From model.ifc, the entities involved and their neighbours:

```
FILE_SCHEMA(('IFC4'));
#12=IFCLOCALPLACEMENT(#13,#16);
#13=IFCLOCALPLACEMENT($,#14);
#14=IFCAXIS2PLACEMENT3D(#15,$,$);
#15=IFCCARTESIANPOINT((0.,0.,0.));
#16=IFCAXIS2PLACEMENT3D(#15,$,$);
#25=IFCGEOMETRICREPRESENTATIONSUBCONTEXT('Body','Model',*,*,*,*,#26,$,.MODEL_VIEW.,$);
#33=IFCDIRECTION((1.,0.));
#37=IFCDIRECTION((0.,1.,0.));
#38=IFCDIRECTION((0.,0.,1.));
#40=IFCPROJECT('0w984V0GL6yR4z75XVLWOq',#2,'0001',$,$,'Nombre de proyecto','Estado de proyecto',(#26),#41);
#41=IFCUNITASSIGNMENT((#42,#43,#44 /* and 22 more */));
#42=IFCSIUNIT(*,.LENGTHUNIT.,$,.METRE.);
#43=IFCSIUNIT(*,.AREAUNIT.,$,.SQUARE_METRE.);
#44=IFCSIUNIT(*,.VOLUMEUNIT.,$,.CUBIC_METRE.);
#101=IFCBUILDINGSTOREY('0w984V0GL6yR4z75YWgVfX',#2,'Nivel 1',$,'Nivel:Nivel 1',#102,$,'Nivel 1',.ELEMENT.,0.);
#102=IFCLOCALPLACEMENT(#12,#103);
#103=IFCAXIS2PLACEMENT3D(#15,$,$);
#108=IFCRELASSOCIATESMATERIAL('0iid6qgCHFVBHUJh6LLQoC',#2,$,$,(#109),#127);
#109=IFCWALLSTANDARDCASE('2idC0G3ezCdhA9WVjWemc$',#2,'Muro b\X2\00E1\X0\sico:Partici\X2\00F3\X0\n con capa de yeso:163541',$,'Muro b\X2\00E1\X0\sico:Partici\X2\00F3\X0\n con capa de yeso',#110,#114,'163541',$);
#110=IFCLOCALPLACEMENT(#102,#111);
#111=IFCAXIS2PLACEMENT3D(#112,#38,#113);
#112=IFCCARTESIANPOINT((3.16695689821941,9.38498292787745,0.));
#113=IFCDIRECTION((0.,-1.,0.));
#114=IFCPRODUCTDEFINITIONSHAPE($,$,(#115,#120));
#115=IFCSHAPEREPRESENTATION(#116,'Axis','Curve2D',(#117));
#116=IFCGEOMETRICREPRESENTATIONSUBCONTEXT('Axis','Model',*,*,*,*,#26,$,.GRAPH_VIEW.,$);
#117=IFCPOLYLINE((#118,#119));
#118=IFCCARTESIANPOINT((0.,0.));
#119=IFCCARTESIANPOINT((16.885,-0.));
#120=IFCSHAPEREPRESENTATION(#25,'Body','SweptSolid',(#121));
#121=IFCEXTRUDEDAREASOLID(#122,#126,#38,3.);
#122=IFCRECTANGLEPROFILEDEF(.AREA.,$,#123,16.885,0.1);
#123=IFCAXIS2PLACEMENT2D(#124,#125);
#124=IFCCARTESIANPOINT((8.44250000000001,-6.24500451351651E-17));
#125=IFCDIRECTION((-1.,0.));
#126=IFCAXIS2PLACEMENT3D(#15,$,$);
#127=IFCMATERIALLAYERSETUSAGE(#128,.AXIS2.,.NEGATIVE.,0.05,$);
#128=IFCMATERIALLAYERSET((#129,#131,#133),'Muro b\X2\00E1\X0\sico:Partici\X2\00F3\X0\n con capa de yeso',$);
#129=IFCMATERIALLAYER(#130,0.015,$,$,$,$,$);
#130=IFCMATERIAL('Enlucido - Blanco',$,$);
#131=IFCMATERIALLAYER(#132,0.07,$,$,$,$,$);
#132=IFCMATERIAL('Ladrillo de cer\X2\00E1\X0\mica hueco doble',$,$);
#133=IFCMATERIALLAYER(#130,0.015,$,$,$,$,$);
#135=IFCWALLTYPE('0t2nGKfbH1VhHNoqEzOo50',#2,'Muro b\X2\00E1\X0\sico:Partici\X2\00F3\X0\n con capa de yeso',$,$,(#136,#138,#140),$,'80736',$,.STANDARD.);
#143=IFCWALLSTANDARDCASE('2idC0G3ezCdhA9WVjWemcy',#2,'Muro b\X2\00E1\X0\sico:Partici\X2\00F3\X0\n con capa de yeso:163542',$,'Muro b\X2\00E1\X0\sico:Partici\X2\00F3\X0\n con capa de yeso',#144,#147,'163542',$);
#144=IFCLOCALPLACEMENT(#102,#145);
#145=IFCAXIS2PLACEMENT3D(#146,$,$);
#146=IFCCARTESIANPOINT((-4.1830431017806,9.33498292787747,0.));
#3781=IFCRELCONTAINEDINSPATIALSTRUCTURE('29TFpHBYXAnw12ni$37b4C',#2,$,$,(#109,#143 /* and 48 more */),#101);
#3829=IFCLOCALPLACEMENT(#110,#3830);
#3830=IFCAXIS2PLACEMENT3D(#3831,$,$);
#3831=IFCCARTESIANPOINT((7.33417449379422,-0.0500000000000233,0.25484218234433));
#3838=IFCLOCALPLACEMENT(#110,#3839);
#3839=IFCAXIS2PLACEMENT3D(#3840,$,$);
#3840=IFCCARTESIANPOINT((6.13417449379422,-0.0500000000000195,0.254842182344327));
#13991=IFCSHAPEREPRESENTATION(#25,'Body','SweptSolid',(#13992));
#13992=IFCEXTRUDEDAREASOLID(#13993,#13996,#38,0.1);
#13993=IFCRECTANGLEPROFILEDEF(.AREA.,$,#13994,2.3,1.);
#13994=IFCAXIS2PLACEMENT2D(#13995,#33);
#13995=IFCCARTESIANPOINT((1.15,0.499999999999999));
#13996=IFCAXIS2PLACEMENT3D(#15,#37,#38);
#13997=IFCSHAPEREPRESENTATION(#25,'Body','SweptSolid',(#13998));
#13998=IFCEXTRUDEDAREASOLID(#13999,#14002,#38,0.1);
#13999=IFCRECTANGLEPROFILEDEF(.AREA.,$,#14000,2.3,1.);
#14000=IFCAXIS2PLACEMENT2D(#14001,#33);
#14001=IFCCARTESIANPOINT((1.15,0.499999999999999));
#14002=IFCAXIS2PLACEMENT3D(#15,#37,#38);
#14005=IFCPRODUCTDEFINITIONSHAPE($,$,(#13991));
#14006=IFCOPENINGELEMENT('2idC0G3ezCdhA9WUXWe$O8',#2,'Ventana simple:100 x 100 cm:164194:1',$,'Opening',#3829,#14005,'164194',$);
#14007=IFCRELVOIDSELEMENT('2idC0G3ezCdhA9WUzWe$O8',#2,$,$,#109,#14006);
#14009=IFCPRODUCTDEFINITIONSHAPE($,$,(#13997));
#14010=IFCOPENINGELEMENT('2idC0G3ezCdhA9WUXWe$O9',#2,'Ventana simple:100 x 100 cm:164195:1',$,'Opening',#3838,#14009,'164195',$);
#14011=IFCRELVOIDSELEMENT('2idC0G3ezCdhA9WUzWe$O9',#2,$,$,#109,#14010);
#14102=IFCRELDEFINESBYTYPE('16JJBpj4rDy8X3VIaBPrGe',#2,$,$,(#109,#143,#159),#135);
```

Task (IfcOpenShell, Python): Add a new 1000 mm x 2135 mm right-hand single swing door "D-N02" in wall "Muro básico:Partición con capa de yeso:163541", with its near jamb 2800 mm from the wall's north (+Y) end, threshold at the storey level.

```python
import numpy as np
import ifcopenshell
import ifcopenshell.api.feature
import ifcopenshell.api.geometry
import ifcopenshell.api.root
import ifcopenshell.api.spatial
import ifcopenshell.geom
import ifcopenshell.util.element
import ifcopenshell.util.placement
import ifcopenshell.util.representation
import ifcopenshell.util.shape
import ifcopenshell.util.unit

model = ifcopenshell.open("model.ifc")
unit_scale = ifcopenshell.util.unit.calculate_unit_scale(model)
settings = ifcopenshell.geom.settings()


def volume(element):
    """Net volume in cubic metres, openings subtracted."""
    shape = ifcopenshell.geom.create_shape(settings, element)
    return ifcopenshell.util.shape.get_volume(shape.geometry)


wall = model.by_id(109)
storey = ifcopenshell.util.element.get_container(wall, ifc_class="IfcBuildingStorey")
context = ifcopenshell.util.representation.get_context(model, "Model", "Body", "MODEL_VIEW")
before = volume(wall)

width, height, from_end, sill = 1, 2.135, 2.8, 0.0  # metres

# The wall runs along its own X axis, and the end named is its -X end.
wall_shape = ifcopenshell.geom.create_shape(settings, wall)
x, y, z = ifcopenshell.util.shape.get_vertices(wall_shape.geometry).T
start = x.min() + from_end
face, thickness = float(y.min()), float(y.max() - y.min())
wall_matrix = ifcopenshell.util.placement.get_local_placement(wall.ObjectPlacement)
level = ifcopenshell.util.placement.get_local_placement(storey.ObjectPlacement)[2, 3]


def in_wall(x, y):
    """Placement at x, y metres in the wall's axes, at sill height."""
    matrix = wall_matrix.copy()
    matrix[:, 3] = wall_matrix @ np.array([x / unit_scale, y / unit_scale, 0.0, 1.0])
    matrix[2, 3] = level + sill / unit_scale
    return matrix


# Opening: a box that overshoots both wall faces by 50 mm.
opening = ifcopenshell.api.root.create_entity(model, ifc_class="IfcOpeningElement", predefined_type="OPENING")
box = ifcopenshell.api.geometry.add_wall_representation(
    model, context=context, length=width, height=height, thickness=thickness + 0.1
)
ifcopenshell.api.geometry.assign_representation(model, product=opening, representation=box)
ifcopenshell.api.geometry.edit_object_placement(model, product=opening, matrix=in_wall(start, face - 0.05), is_si=False)
ifcopenshell.api.feature.add_feature(model, feature=opening, element=wall)

door = ifcopenshell.api.root.create_entity(model, ifc_class="IfcDoor", name="D-N02", predefined_type="DOOR")
door.OverallWidth, door.OverallHeight = width / unit_scale, height / unit_scale
door.OperationType = "SINGLE_SWING_RIGHT"
body = ifcopenshell.api.geometry.add_door_representation(
    model,
    context=context,
    overall_width=door.OverallWidth,
    overall_height=door.OverallHeight,
    operation_type="SINGLE_SWING_RIGHT",
    lining_properties={"LiningDepth": thickness / unit_scale, "ThresholdDepth": thickness / unit_scale},
)
ifcopenshell.api.geometry.assign_representation(model, product=door, representation=body)
ifcopenshell.api.spatial.assign_container(model, products=[door], relating_structure=storey)
ifcopenshell.api.feature.add_filling(model, opening=opening, element=door)

# The lining spans the wall, so the door starts at the wall face.
ifcopenshell.api.geometry.edit_object_placement(model, product=door, matrix=in_wall(start, face), is_si=False)

after = volume(wall)

print(f"wall volume {before:.3f} -> {after:.3f} m3")

model.write("model-out.ifc")
```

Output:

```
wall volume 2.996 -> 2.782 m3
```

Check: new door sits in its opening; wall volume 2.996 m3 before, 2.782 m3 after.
